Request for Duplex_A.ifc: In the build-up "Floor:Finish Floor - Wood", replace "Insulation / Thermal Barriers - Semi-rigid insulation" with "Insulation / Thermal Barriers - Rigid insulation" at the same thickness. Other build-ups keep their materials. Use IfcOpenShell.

First a look at what the model holds.

```python
import ifcopenshell
import ifcopenshell.util.element

model = ifcopenshell.open("Duplex_A.ifc")
print(model.schema)
for layer_set in model.by_type("IfcMaterialLayerSet"):
    if layer_set.LayerSetName == "Floor:Finish Floor - Wood":
        for layer in layer_set.MaterialLayers:
            print(layer.id(), layer.Material and layer.Material.Name, layer.LayerThickness, sep=" | ")
        print(len(ifcopenshell.util.element.get_elements_by_material(model, layer_set)), "elements and types use it")
print(sorted(m.Name for m in model.by_type("IfcMaterial") if m.Name)[:60])
```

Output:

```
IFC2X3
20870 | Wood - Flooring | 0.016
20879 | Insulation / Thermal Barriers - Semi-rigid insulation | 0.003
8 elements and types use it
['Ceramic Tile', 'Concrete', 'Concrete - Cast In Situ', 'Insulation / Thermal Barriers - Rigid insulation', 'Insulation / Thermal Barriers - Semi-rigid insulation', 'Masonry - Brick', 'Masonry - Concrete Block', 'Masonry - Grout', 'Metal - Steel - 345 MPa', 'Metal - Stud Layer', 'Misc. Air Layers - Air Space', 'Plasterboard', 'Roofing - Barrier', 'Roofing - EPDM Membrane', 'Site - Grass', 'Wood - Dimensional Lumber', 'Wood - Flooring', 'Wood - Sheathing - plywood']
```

```python
import ifcopenshell
import ifcopenshell.api.material

model = ifcopenshell.open("Duplex_A.ifc")

layer_set = next(s for s in model.by_type("IfcMaterialLayerSet") if s.LayerSetName == "Floor:Finish Floor - Wood")
layer = next(l for l in layer_set.MaterialLayers if l.Material and l.Material.Name == "Insulation / Thermal Barriers - Semi-rigid insulation")
material = next(m for m in model.by_type("IfcMaterial") if m.Name == "Insulation / Thermal Barriers - Rigid insulation")

# Point this one layer at the other material; renaming the old one would change it everywhere.
ifcopenshell.api.material.edit_layer(model, layer=layer, attributes={}, material=material)

print([l.Material.Name if l.Material else None for l in layer_set.MaterialLayers])

model.write("Duplex_A_rev.ifc")
```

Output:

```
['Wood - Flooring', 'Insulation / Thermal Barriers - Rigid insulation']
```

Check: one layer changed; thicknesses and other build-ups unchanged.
